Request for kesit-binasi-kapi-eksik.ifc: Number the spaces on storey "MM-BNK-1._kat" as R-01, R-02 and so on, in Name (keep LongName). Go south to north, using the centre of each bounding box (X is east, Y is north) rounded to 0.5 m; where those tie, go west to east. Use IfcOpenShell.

First a look at what the model holds.

```python
import ifcopenshell
import ifcopenshell.util.element
import ifcopenshell.util.placement

model = ifcopenshell.open("kesit-binasi-kapi-eksik.ifc")
print(model.schema)
storey = next(s for s in model.by_type("IfcBuildingStorey") if s.Name == "MM-BNK-1._kat")
spaces = [e for e in ifcopenshell.util.element.get_decomposition(storey) if e.is_a("IfcSpace")]
for e in sorted(spaces, key=lambda e: e.id()):
    origin = ifcopenshell.util.placement.get_local_placement(e.ObjectPlacement)[:3, 3]
    print(e.id(), e.Name, e.LongName, origin.round(2) + 0.0, sep=" | ")
```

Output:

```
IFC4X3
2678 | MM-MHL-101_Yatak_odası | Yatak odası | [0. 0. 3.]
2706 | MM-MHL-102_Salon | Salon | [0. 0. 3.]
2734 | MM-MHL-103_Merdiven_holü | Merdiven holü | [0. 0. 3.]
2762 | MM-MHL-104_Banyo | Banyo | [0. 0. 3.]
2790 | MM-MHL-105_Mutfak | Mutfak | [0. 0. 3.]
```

```python
import ifcopenshell
import ifcopenshell.geom
import ifcopenshell.util.element
import ifcopenshell.util.shape

model = ifcopenshell.open("kesit-binasi-kapi-eksik.ifc")
settings = ifcopenshell.geom.settings()
settings.set("use-world-coords", True)


def centre(element):
    shape = ifcopenshell.geom.create_shape(settings, element)
    return ifcopenshell.util.shape.get_bbox_centroid(shape.geometry)


storey = next(s for s in model.by_type("IfcBuildingStorey") if s.Name == "MM-BNK-1._kat")
spaces = [e for e in ifcopenshell.util.element.get_decomposition(storey) if e.is_a("IfcSpace")]

# Insertion points can sit at a corner or the storey origin, so sort by the geometry (in metres).
centres = {e: centre(e) for e in spaces}
spaces.sort(key=lambda e: (round(centres[e][1] / 0.5), centres[e][0]))

for i, e in enumerate(spaces, start=1):
    number = f"R-{i:02d}"
    e.Name = number
    print(e.id(), number)

model.write("kesit-binasi-kapi-eksik_updated.ifc")
```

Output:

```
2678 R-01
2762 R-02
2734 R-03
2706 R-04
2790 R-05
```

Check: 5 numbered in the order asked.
